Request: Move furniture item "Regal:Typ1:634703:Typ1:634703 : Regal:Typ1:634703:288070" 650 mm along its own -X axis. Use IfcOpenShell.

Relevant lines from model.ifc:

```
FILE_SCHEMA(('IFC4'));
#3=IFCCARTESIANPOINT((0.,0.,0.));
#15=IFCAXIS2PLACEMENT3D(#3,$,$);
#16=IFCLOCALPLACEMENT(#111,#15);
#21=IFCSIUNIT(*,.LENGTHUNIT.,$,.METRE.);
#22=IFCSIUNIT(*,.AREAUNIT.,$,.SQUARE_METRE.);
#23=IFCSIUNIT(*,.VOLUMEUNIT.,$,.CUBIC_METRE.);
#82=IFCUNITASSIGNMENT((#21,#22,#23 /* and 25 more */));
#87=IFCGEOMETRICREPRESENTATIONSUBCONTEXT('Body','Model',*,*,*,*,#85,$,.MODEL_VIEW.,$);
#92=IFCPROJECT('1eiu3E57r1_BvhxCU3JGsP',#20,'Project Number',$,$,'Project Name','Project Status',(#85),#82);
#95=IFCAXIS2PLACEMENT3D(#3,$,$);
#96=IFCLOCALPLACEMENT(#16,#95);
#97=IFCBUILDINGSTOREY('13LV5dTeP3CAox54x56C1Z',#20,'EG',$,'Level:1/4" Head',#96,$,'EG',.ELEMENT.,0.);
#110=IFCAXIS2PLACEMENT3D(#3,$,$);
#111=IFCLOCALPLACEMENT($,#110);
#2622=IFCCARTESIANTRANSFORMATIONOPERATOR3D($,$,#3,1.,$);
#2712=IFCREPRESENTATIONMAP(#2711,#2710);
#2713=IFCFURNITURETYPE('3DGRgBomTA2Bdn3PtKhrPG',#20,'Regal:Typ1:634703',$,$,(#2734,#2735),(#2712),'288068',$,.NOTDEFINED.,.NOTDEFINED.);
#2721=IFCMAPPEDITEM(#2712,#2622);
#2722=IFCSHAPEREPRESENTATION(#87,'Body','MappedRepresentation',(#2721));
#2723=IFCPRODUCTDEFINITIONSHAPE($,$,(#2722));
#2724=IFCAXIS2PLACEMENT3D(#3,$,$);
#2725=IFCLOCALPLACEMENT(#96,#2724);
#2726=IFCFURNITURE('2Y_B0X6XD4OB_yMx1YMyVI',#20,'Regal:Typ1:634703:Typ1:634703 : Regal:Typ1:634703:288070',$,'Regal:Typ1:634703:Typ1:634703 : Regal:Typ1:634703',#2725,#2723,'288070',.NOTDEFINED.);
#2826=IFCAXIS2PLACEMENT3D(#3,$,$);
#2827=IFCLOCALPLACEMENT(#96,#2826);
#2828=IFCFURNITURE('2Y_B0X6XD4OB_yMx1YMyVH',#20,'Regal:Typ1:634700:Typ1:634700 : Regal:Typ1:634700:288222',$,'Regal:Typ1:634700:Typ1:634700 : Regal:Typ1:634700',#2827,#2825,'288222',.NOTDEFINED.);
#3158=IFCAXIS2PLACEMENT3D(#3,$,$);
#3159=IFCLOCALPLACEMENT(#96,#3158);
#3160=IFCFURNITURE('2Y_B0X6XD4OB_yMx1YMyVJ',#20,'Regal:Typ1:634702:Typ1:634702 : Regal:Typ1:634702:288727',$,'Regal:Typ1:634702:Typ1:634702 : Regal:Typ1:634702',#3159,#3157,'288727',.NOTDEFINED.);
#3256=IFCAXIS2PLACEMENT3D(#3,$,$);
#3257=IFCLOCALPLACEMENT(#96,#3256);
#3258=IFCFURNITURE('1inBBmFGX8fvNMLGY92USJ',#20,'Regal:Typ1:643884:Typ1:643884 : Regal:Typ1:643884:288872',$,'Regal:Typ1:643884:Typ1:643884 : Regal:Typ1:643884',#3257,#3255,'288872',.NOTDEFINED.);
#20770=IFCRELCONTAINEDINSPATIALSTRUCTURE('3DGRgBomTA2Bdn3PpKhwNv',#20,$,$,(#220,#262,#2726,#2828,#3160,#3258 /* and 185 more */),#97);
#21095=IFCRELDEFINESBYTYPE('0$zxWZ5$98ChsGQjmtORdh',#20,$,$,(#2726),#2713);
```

```python
import ifcopenshell
import ifcopenshell.api.geometry
import ifcopenshell.util.placement
import ifcopenshell.util.unit

model = ifcopenshell.open("model.ifc")
unit_scale = ifcopenshell.util.unit.calculate_unit_scale(model)

item = model.by_guid("2Y_B0X6XD4OB_yMx1YMyVI")
matrix = ifcopenshell.util.placement.get_local_placement(item.ObjectPlacement)
matrix[:3, 3] -= matrix[:3, 0] * 0.65 / unit_scale
ifcopenshell.api.geometry.edit_object_placement(model, product=item, matrix=matrix, is_si=False)

print(ifcopenshell.util.placement.get_local_placement(item.ObjectPlacement).round(3) + 0.0)

model.write("model_rev.ifc")
```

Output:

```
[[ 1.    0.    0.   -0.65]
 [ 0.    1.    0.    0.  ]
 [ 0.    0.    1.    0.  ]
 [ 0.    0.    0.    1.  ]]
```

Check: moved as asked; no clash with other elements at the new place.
